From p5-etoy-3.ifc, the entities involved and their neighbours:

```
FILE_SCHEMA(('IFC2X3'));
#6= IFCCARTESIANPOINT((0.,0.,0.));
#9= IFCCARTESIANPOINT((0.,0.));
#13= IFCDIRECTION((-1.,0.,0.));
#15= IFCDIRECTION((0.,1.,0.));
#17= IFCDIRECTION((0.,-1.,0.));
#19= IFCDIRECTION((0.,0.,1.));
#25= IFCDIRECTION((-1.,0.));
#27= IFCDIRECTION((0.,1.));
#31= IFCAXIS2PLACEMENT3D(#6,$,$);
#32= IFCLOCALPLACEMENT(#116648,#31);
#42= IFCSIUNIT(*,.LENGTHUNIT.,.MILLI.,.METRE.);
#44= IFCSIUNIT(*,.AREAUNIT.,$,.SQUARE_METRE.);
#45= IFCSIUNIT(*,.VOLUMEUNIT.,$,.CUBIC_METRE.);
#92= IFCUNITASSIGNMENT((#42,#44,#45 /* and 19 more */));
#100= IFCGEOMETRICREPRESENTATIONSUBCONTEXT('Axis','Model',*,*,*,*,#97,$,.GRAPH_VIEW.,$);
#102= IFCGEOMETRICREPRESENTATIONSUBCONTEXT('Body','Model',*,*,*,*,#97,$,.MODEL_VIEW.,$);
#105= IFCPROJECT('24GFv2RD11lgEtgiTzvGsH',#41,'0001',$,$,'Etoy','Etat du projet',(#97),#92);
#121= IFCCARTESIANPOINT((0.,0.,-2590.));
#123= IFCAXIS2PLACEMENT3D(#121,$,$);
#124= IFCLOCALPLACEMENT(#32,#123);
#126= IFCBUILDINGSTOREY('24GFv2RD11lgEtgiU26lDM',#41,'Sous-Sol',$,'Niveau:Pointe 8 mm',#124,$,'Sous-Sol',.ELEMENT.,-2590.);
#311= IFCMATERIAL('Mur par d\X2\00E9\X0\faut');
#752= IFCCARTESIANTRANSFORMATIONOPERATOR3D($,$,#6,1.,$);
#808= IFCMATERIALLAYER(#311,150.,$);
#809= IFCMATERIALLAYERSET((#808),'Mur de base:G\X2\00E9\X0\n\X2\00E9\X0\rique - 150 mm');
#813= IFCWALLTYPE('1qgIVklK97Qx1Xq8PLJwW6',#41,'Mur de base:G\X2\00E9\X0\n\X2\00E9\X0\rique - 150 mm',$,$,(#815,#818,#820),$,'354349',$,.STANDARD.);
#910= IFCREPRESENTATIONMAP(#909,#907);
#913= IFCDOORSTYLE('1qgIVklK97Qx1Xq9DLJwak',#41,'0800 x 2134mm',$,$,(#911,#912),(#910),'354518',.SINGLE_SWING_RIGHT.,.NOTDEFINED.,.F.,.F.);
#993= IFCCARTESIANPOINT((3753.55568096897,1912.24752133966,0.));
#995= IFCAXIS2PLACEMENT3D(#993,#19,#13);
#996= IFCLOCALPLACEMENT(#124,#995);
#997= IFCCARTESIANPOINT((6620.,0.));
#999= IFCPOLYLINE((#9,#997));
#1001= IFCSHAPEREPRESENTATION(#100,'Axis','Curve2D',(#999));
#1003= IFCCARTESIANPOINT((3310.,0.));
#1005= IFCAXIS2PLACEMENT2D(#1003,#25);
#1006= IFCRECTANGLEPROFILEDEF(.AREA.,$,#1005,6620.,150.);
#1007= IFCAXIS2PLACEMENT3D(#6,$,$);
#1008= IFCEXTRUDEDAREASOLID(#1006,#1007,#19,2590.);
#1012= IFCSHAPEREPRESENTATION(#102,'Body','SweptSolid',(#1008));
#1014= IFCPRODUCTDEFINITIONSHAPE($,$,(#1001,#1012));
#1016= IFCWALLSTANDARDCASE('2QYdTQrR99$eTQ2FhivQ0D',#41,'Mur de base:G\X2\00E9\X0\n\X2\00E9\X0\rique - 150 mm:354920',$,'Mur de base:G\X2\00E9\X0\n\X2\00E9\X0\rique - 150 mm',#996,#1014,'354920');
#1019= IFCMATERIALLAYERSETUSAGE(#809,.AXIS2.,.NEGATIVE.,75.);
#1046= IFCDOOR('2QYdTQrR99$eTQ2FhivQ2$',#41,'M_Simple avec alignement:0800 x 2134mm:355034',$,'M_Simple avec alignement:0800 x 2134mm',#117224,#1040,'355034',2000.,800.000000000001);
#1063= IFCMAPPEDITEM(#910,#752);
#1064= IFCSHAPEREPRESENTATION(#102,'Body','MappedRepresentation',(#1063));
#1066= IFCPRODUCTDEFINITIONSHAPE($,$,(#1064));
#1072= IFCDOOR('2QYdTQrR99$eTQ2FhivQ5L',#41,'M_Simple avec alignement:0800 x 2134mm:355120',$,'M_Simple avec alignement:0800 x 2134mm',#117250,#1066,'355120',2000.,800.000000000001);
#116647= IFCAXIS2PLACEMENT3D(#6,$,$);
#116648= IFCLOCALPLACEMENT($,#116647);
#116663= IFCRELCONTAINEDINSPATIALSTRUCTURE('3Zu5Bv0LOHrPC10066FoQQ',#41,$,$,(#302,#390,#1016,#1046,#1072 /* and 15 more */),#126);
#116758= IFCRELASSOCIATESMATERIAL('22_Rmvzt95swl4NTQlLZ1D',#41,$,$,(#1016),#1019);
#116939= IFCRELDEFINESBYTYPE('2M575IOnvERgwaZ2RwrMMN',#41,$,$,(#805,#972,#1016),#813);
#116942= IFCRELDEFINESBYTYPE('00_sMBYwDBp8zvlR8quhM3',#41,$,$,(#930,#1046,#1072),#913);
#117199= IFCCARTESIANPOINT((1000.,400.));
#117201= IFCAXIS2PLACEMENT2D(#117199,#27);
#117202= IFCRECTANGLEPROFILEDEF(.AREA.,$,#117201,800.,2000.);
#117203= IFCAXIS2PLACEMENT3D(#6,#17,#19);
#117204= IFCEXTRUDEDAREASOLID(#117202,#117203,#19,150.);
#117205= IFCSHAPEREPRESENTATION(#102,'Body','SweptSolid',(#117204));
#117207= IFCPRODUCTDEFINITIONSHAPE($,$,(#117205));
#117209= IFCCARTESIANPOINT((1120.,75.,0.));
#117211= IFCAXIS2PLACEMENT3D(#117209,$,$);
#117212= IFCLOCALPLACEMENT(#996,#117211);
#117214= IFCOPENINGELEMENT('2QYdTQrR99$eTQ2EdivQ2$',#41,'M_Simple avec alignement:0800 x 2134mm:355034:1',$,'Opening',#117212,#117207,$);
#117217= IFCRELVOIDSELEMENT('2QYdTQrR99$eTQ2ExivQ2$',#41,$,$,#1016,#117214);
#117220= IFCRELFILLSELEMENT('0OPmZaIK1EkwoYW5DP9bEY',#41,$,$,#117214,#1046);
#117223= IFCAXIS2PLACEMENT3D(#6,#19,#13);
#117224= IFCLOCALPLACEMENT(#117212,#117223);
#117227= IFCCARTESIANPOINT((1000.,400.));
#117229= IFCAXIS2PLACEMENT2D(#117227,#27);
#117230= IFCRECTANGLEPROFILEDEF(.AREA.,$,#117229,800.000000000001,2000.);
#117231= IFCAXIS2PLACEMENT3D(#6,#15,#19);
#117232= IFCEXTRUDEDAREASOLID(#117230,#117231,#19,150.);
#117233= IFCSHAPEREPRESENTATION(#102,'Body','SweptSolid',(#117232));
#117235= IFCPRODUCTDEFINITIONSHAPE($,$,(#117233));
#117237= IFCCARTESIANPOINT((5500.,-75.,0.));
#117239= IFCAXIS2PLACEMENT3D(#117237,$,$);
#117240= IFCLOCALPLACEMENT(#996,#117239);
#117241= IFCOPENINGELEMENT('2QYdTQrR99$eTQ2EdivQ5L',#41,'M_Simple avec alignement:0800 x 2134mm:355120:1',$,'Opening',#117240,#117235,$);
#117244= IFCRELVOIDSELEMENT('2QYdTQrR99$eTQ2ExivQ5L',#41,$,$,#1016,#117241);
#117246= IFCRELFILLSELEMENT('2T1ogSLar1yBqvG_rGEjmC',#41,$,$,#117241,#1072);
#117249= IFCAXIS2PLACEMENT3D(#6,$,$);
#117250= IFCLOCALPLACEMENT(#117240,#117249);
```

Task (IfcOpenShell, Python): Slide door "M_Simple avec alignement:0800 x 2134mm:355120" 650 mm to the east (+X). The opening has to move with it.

```python
import ifcopenshell
import ifcopenshell.api.geometry
import ifcopenshell.util.placement
import ifcopenshell.util.unit

model = ifcopenshell.open("p5-etoy-3.ifc")
unit_scale = ifcopenshell.util.unit.calculate_unit_scale(model)

door = model.by_guid("2QYdTQrR99$eTQ2FhivQ5L")
opening = door.FillsVoids[0].RelatingOpeningElement
wall = opening.VoidsElements[0].RelatingBuildingElement

wall_matrix = ifcopenshell.util.placement.get_local_placement(wall.ObjectPlacement)
shift = wall_matrix[:3, 0] * -0.65 / unit_scale
before = ifcopenshell.util.placement.get_local_placement(door.ObjectPlacement)[:3, 3].copy()

# The door is placed relative to its opening, so it follows when the opening moves.
matrix = ifcopenshell.util.placement.get_local_placement(opening.ObjectPlacement)
matrix[:3, 3] += shift
ifcopenshell.api.geometry.edit_object_placement(
    model, product=opening, matrix=matrix, is_si=False, should_transform_children=True
)

after = ifcopenshell.util.placement.get_local_placement(door.ObjectPlacement)[:3, 3]
print("door moved by", (after - before).round(3) + 0.0)

model.write("p5-etoy-3_rev.ifc")
```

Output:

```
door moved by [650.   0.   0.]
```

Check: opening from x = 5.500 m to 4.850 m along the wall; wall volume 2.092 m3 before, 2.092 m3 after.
